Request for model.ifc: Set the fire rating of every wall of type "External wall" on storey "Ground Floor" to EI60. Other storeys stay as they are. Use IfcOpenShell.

First a look at what the model holds.

```python
import ifcopenshell
import ifcopenshell.util.element

model = ifcopenshell.open("model.ifc")
print(model.schema)
storey = next(s for s in model.by_type("IfcBuildingStorey") if s.Name == "Ground Floor")
walls = [e for e in ifcopenshell.util.element.get_decomposition(storey) if e.is_a("IfcWall")]
seen = {}
for e in walls:
    element_type = ifcopenshell.util.element.get_type(e)
    key = (element_type.Name if element_type != e and element_type else None, ifcopenshell.util.element.get_pset(e, "Pset_WallCommon", "FireRating"))
    seen[key] = seen.get(key, 0) + 1
for (name, value), count in sorted(seen.items(), key=str):
    print(count, "x", name, "|", value)
```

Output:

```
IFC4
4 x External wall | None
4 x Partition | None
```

```python
import ifcopenshell
import ifcopenshell.api.pset
import ifcopenshell.util.element

model = ifcopenshell.open("model.ifc")

storey = next(s for s in model.by_type("IfcBuildingStorey") if s.Name == "Ground Floor")
walls = [e for e in ifcopenshell.util.element.get_decomposition(storey) if e.is_a("IfcWall")]

count = 0
for e in walls:
    element_type = ifcopenshell.util.element.get_type(e)
    if element_type in (None, e) or element_type.Name != "External wall":
        continue
    # add_pset returns the element's existing set when there is one.
    pset = ifcopenshell.api.pset.add_pset(model, product=e, name="Pset_WallCommon")
    ifcopenshell.api.pset.edit_pset(model, pset=pset, properties={"FireRating": "EI60"})
    count += 1

print(count, "walls updated")

model.write("model-out.ifc")
```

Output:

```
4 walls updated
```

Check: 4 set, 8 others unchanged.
